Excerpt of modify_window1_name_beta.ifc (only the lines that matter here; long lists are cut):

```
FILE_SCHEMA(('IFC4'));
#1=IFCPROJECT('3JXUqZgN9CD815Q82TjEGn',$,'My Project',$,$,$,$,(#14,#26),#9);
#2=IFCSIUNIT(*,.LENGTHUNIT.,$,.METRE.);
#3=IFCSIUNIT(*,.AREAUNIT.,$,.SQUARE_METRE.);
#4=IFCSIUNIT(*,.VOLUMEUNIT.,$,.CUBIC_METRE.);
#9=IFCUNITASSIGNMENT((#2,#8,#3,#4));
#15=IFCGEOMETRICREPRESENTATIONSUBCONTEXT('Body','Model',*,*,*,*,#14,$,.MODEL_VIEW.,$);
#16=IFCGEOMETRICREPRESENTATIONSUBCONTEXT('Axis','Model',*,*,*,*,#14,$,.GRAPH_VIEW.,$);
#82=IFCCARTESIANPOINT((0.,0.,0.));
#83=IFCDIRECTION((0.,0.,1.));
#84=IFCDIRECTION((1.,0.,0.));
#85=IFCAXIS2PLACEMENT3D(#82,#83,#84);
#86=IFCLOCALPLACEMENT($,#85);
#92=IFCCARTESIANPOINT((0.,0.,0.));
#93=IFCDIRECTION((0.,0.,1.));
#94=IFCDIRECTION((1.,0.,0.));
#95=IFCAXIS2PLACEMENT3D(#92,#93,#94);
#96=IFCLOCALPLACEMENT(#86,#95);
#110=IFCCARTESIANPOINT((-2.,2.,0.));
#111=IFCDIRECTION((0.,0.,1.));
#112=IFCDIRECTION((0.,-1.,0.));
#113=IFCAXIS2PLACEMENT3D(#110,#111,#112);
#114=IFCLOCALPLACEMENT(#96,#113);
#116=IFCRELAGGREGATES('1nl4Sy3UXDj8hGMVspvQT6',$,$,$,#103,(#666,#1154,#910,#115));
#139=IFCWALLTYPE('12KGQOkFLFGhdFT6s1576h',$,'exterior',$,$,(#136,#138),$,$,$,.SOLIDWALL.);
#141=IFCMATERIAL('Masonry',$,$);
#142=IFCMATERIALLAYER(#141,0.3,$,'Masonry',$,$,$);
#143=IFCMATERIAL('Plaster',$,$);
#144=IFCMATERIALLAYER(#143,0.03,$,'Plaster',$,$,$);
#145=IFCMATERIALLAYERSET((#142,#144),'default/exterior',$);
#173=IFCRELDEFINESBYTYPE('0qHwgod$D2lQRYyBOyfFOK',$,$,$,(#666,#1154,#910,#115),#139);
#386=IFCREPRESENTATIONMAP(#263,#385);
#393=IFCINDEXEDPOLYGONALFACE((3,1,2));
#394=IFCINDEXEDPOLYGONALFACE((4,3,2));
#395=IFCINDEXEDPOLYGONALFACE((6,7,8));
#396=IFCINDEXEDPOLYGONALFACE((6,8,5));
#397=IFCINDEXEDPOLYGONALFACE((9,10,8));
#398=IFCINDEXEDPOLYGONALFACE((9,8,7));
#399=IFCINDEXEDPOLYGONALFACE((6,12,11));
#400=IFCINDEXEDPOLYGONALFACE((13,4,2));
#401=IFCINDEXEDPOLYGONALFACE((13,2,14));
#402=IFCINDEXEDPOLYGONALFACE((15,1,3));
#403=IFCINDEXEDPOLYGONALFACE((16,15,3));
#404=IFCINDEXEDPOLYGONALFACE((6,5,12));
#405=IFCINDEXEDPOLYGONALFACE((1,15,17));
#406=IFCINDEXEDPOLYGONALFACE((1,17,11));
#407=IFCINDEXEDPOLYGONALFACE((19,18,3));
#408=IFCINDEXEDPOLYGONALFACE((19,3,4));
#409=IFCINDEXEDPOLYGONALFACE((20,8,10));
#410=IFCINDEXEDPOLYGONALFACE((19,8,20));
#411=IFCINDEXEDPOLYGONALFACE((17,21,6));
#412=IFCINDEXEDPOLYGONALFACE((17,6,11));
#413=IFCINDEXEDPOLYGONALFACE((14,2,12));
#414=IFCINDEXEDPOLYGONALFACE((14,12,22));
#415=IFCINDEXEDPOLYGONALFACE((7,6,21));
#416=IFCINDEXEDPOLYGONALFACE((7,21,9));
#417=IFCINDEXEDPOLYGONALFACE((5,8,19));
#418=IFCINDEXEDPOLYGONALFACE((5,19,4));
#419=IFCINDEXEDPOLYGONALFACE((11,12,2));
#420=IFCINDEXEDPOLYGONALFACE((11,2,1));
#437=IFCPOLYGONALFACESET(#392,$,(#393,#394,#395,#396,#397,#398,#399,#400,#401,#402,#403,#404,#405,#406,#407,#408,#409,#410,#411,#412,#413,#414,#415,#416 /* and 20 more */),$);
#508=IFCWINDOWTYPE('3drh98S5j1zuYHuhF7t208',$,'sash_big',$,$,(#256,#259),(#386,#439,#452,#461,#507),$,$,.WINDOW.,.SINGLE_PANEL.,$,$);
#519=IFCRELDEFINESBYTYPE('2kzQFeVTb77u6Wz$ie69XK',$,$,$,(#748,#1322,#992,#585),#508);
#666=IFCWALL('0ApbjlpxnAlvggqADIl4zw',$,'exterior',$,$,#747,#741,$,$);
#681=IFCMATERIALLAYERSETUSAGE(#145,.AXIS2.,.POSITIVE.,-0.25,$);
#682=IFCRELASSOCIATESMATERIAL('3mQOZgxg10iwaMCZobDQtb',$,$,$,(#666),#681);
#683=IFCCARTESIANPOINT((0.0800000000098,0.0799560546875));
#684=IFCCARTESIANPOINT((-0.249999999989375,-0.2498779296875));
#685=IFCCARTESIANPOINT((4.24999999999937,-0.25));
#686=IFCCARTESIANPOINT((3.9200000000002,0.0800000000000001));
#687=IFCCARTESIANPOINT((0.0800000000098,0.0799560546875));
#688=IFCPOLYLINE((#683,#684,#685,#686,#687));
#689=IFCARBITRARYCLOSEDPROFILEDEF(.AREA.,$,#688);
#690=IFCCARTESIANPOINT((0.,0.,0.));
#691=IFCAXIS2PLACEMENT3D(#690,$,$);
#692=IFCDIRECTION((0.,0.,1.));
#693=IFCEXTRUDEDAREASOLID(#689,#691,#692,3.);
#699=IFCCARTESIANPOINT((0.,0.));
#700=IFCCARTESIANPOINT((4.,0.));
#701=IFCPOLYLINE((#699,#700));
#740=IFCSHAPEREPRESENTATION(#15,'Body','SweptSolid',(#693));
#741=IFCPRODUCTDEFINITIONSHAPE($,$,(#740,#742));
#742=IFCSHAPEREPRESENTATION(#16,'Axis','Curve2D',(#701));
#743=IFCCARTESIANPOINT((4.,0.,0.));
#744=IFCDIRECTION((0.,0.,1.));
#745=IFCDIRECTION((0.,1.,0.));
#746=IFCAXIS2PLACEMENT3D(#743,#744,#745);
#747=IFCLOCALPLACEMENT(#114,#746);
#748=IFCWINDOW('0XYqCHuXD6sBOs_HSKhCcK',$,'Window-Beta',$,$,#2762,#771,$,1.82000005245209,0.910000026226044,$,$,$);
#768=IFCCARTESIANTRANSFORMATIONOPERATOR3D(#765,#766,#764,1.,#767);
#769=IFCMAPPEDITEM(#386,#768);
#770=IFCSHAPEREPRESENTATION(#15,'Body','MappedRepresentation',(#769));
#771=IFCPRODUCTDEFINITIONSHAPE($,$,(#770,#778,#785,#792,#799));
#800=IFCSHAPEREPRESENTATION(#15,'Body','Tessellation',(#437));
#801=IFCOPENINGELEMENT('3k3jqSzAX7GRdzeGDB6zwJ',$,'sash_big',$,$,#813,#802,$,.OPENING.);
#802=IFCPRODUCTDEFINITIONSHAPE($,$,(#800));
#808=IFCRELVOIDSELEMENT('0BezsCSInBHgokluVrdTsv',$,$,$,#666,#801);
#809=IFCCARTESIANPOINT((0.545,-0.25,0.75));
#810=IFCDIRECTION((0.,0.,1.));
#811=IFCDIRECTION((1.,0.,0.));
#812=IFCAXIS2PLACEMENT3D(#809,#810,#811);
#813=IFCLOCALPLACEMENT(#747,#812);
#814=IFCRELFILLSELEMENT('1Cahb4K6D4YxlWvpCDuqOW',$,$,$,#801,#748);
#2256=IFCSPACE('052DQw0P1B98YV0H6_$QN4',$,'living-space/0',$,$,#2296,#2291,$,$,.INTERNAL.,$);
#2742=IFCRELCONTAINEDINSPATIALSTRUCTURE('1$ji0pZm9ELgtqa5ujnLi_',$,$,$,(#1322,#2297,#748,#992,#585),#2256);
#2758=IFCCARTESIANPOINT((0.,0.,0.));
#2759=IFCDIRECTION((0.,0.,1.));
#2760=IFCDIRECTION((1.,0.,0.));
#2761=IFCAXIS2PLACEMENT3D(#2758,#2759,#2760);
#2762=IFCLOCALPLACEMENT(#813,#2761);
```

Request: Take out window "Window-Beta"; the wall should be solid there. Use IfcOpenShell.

```python
import ifcopenshell
import ifcopenshell.api.feature
import ifcopenshell.api.root
import ifcopenshell.geom
import ifcopenshell.util.shape

model = ifcopenshell.open("modify_window1_name_beta.ifc")
settings = ifcopenshell.geom.settings()


def volume(element):
    """Net volume in cubic metres, openings subtracted."""
    shape = ifcopenshell.geom.create_shape(settings, element)
    return ifcopenshell.util.shape.get_volume(shape.geometry)


window = model.by_guid("0XYqCHuXD6sBOs_HSKhCcK")
opening = window.FillsVoids[0].RelatingOpeningElement
wall = opening.VoidsElements[0].RelatingBuildingElement
before = volume(wall)

ifcopenshell.api.root.remove_product(model, product=window)
ifcopenshell.api.feature.remove_feature(model, feature=opening)

after = volume(wall)

print(f"wall volume {before:.3f} -> {after:.3f} m3")

model.write("modify_window1_name_beta_updated.ifc")
```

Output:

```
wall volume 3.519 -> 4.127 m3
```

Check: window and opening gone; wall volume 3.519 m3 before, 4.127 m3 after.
